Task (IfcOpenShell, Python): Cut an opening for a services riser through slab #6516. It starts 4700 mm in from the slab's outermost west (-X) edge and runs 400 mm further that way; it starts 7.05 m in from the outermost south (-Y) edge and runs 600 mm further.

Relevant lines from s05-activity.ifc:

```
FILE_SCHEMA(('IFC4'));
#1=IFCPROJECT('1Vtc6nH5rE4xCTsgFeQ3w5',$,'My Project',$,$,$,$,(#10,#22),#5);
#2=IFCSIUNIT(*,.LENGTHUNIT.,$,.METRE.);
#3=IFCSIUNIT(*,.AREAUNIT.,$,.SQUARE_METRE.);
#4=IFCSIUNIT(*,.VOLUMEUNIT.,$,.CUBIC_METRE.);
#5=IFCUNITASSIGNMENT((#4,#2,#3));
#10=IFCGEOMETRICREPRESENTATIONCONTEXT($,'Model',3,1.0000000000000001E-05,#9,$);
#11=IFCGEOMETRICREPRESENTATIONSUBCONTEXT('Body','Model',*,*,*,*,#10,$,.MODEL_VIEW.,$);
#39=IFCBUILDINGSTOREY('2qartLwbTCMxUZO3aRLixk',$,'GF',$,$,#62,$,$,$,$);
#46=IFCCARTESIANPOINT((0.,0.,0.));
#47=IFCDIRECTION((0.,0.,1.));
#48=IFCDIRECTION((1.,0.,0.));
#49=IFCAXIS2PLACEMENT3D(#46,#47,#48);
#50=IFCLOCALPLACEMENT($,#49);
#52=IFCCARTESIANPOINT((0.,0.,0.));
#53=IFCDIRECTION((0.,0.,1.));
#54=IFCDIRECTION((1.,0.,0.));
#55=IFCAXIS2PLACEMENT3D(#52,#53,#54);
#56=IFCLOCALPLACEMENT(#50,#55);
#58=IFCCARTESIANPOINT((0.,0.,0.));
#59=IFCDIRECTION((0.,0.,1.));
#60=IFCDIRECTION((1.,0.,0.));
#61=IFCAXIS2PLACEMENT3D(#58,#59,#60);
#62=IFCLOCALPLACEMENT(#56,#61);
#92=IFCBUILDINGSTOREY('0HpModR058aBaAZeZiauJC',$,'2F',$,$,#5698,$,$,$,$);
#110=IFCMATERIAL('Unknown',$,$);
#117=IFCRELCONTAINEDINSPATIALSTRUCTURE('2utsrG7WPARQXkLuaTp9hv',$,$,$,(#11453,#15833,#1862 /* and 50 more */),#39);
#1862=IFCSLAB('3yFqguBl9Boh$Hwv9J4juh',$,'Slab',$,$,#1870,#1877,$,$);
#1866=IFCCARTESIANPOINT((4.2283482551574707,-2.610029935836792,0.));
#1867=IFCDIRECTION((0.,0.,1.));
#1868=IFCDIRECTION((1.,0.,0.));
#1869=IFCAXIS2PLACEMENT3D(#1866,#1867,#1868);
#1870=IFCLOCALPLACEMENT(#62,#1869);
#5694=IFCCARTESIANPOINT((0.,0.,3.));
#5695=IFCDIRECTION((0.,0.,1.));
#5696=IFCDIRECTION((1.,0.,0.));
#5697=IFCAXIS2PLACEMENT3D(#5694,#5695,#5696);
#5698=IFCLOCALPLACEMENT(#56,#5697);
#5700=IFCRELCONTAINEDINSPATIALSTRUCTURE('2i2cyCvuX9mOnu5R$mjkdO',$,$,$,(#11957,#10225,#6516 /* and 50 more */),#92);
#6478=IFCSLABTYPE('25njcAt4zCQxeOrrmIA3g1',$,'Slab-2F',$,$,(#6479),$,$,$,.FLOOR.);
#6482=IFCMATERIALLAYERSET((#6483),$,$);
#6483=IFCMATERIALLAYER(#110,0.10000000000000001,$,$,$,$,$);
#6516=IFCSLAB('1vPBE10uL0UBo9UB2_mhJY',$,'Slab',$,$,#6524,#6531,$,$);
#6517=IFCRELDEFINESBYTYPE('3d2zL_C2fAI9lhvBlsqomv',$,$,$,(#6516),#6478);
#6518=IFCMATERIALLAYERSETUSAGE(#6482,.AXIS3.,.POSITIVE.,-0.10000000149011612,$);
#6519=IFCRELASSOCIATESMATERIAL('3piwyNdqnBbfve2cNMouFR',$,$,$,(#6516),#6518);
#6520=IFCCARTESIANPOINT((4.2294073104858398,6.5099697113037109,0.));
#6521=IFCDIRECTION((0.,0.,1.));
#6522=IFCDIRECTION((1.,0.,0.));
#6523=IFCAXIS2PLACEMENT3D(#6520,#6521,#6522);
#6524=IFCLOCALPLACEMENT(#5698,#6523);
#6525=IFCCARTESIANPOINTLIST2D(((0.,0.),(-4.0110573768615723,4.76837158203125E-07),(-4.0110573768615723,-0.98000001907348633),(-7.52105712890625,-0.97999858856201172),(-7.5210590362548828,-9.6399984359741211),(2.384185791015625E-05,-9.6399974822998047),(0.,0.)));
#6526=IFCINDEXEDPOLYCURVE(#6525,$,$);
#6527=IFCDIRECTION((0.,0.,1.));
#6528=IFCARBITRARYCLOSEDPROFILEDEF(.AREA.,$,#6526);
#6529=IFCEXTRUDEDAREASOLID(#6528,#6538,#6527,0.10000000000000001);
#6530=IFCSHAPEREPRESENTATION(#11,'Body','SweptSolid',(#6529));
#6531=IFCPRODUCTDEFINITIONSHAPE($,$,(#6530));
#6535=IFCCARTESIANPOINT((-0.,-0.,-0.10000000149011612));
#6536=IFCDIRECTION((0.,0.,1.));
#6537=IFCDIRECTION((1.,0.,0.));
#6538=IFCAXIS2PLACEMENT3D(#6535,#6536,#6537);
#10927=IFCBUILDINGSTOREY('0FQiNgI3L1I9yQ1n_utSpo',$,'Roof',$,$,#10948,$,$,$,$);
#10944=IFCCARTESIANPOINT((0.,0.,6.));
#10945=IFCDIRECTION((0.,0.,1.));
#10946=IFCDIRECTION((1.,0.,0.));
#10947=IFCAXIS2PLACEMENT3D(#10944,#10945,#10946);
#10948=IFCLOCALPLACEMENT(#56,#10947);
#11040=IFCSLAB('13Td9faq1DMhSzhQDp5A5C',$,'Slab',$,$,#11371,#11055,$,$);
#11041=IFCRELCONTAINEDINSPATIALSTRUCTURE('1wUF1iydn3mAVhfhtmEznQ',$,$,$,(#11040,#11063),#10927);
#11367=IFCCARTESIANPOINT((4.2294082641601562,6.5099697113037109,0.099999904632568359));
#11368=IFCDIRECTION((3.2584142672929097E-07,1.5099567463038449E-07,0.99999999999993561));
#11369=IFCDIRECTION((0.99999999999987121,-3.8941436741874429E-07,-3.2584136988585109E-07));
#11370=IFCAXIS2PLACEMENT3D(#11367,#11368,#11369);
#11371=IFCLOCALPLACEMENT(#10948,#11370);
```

```python
import numpy as np
import ifcopenshell
import ifcopenshell.api.feature
import ifcopenshell.api.geometry
import ifcopenshell.api.root
import ifcopenshell.geom
import ifcopenshell.util.placement
import ifcopenshell.util.representation
import ifcopenshell.util.shape
import ifcopenshell.util.unit

model = ifcopenshell.open("s05-activity.ifc")
unit_scale = ifcopenshell.util.unit.calculate_unit_scale(model)
settings = ifcopenshell.geom.settings()


def volume(element):
    """Net volume in cubic metres, openings subtracted."""
    shape = ifcopenshell.geom.create_shape(settings, element)
    return ifcopenshell.util.shape.get_volume(shape.geometry)


slab = model.by_id(6516)
before = volume(slab)

# Extent in the slab's own axes, in metres. The edges named are its -X and -Y sides.
slab_shape = ifcopenshell.geom.create_shape(settings, slab)
vertices = ifcopenshell.util.shape.get_vertices(slab_shape.geometry)
x_min, y_min, bottom = vertices.min(axis=0)
top = vertices[:, 2].max()

opening = ifcopenshell.api.root.create_entity(model, ifc_class="IfcOpeningElement", name="Services riser opening", predefined_type="OPENING")
context = ifcopenshell.util.representation.get_context(model, "Model", "Body", "MODEL_VIEW")
width, depth = 0.4, 0.6
outline = [(0.0, 0.0), (width, 0.0), (width, depth), (0.0, depth), (0.0, 0.0)]
# Overshoot both faces by 50 mm so the cut is clean.
shape = ifcopenshell.api.geometry.add_slab_representation(
    model, context=context, depth=top - bottom + 0.1, polyline=outline
)
ifcopenshell.api.geometry.assign_representation(model, product=opening, representation=shape)

matrix = ifcopenshell.util.placement.get_local_placement(slab.ObjectPlacement)
matrix[:, 3] = matrix @ np.append(np.array([x_min + 4.7, y_min + 7.05, bottom - 0.05]) / unit_scale, 1.0)
ifcopenshell.api.geometry.edit_object_placement(model, product=opening, matrix=matrix, is_si=False)
ifcopenshell.api.feature.add_feature(model, feature=opening, element=slab)

after = volume(slab)

print(f"slab volume {before:.3f} -> {after:.3f} m3")

model.write("s05-activity_updated.ifc")
```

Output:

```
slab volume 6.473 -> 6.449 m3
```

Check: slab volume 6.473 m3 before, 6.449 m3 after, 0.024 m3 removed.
